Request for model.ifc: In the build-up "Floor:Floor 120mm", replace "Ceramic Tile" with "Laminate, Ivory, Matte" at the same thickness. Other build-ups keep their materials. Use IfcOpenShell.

First a look at what the model holds.

```python
import ifcopenshell
import ifcopenshell.util.element

model = ifcopenshell.open("model.ifc")
print(model.schema)
for layer_set in model.by_type("IfcMaterialLayerSet"):
    if layer_set.LayerSetName == "Floor:Floor 120mm":
        for layer in layer_set.MaterialLayers:
            print(layer.id(), layer.Material and layer.Material.Name, layer.LayerThickness, sep=" | ")
        print(len(ifcopenshell.util.element.get_elements_by_material(model, layer_set)), "elements and types use it")
print(sorted(m.Name for m in model.by_type("IfcMaterial") if m.Name)[:60])
```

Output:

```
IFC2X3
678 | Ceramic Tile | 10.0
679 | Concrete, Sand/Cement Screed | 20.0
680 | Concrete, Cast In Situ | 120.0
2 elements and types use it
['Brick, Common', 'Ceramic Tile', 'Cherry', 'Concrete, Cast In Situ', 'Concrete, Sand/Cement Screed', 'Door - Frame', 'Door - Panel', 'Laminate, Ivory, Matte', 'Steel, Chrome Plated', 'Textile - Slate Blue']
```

```python
import ifcopenshell
import ifcopenshell.api.material

model = ifcopenshell.open("model.ifc")

layer_set = next(s for s in model.by_type("IfcMaterialLayerSet") if s.LayerSetName == "Floor:Floor 120mm")
layer = next(l for l in layer_set.MaterialLayers if l.Material and l.Material.Name == "Ceramic Tile")
material = next(m for m in model.by_type("IfcMaterial") if m.Name == "Laminate, Ivory, Matte")

# Point this one layer at the other material; renaming the old one would change it everywhere.
ifcopenshell.api.material.edit_layer(model, layer=layer, attributes={}, material=material)

print([l.Material.Name if l.Material else None for l in layer_set.MaterialLayers])

model.write("model_v2.ifc")
```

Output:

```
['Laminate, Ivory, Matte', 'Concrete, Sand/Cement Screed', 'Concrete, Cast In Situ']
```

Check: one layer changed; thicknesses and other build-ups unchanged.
